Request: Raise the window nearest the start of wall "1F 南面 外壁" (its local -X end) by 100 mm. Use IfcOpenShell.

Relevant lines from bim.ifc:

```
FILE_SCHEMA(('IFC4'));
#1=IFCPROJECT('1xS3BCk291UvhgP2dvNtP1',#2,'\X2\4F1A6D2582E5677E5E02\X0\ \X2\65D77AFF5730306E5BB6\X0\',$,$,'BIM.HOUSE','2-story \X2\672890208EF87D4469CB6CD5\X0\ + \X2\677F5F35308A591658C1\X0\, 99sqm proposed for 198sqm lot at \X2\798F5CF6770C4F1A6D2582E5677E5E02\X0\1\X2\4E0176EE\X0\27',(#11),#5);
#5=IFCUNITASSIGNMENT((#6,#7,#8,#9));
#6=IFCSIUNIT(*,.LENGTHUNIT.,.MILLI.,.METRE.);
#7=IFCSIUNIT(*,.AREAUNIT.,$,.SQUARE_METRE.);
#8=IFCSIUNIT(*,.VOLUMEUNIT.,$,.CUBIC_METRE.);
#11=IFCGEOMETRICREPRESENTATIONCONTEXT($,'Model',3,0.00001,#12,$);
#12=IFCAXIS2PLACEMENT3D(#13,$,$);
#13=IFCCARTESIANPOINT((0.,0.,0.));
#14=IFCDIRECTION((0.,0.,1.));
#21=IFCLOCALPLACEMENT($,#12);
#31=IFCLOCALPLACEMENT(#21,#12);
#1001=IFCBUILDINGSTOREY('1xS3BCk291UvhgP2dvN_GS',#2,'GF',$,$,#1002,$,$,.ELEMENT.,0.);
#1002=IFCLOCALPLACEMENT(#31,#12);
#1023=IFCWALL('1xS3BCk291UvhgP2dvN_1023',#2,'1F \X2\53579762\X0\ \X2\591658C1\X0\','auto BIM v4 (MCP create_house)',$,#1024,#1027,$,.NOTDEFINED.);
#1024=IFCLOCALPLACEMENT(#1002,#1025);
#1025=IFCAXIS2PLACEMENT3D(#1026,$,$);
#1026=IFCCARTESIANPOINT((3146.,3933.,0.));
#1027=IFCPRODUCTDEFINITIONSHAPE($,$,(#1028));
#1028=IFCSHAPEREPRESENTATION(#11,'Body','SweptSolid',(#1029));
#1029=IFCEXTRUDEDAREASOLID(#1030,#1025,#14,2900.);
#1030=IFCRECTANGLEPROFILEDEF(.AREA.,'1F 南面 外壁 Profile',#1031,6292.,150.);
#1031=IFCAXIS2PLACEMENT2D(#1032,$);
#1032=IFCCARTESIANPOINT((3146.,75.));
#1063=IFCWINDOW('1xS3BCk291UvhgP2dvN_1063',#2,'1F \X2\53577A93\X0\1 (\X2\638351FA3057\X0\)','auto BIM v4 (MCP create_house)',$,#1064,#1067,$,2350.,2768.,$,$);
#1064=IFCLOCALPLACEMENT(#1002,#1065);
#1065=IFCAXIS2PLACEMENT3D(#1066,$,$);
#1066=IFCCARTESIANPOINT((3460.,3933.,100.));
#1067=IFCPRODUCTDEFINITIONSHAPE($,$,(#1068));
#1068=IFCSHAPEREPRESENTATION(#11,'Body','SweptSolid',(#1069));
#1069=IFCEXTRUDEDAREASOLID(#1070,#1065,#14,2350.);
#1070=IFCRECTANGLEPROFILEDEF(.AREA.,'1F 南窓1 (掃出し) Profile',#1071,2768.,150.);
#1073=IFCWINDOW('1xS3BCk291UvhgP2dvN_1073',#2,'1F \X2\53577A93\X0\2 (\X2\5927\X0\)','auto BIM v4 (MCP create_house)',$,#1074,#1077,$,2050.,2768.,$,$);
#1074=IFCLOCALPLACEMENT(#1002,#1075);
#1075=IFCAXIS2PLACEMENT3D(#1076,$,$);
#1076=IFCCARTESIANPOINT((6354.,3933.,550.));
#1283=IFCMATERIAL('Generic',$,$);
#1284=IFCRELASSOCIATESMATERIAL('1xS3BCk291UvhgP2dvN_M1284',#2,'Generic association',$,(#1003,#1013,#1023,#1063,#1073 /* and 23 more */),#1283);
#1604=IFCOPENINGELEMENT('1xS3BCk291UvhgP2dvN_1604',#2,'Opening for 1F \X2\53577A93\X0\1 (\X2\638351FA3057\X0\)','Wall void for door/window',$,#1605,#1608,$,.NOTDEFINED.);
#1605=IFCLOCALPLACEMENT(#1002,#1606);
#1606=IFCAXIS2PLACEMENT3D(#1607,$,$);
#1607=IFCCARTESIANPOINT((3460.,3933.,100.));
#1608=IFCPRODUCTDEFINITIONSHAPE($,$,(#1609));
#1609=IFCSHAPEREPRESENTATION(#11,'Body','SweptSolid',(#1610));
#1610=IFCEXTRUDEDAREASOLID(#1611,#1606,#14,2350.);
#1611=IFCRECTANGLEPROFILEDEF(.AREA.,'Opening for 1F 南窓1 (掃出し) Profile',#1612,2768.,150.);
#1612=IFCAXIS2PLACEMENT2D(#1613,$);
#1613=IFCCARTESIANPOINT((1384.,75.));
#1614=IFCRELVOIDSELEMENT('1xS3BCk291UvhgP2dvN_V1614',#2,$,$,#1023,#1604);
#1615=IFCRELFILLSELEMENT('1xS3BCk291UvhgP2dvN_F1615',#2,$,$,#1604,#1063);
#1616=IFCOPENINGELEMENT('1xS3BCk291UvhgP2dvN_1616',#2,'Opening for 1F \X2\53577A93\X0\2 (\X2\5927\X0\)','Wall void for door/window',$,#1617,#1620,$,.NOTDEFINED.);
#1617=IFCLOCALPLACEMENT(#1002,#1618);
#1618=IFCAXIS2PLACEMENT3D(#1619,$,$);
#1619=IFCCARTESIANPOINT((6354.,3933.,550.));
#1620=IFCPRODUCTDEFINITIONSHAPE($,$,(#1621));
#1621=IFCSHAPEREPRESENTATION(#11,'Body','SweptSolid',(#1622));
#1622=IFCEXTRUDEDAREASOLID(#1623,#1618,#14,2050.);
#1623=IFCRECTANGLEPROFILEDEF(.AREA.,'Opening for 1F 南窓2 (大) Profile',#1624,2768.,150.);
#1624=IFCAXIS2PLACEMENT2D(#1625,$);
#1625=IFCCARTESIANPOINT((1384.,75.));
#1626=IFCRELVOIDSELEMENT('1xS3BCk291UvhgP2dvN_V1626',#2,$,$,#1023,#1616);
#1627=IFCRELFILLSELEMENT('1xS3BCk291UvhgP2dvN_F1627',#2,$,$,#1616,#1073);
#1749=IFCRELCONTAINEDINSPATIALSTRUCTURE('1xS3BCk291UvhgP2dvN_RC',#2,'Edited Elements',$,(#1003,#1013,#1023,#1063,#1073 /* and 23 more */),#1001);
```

```python
import numpy as np
import ifcopenshell
import ifcopenshell.api.geometry
import ifcopenshell.util.placement
import ifcopenshell.util.unit

model = ifcopenshell.open("bim.ifc")
unit_scale = ifcopenshell.util.unit.calculate_unit_scale(model)

window = model.by_id(1063)
opening = window.FillsVoids[0].RelatingOpeningElement
dz = 100.0

shift = np.array([0.0, 0.0, dz])
# The window is not placed relative to its opening, so move both.
for product in (opening, window):
    matrix = ifcopenshell.util.placement.get_local_placement(product.ObjectPlacement)
    matrix[:3, 3] += shift
    ifcopenshell.api.geometry.edit_object_placement(model, product=product, matrix=matrix, is_si=False)

print(f"moved by {dz * unit_scale:+.3f} m")

model.write("bim_v2.ifc")
```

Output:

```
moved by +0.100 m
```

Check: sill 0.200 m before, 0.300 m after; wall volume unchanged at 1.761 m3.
